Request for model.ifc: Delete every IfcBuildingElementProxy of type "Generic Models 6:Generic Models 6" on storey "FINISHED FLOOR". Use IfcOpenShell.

First a look at what the model holds.

```python
import ifcopenshell
import ifcopenshell.util.element

model = ifcopenshell.open("model.ifc")
print(model.schema)
storey = next(s for s in model.by_type("IfcBuildingStorey") if s.Name == "FINISHED FLOOR")
proxies = [e for e in ifcopenshell.util.element.get_decomposition(storey) if e.is_a("IfcBuildingElementProxy")]
seen = {}
for e in proxies:
    element_type = ifcopenshell.util.element.get_type(e)
    name = element_type.Name if element_type not in (None, e) else None
    seen[name] = seen.get(name, 0) + 1
for name, count in sorted(seen.items(), key=str):
    print(count, "x", name)
```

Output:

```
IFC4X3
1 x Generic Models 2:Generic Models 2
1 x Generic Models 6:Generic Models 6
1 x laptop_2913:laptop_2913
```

```python
import ifcopenshell
import ifcopenshell.api.root
import ifcopenshell.util.element

model = ifcopenshell.open("model.ifc")

storey = next(s for s in model.by_type("IfcBuildingStorey") if s.Name == "FINISHED FLOOR")
proxies = [e for e in ifcopenshell.util.element.get_decomposition(storey) if e.is_a("IfcBuildingElementProxy")]
targets = [e for e in proxies if (t := ifcopenshell.util.element.get_type(e)) not in (None, e) and t.Name == "Generic Models 6:Generic Models 6"]

for e in targets:
    ifcopenshell.api.root.remove_product(model, product=e)
print(len(targets), "removed")

model.write("model-out.ifc")
```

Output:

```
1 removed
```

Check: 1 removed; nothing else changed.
